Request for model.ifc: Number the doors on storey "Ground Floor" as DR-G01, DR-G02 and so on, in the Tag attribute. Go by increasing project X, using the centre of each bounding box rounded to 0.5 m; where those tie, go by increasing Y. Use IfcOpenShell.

First a look at what the model holds.

```python
import ifcopenshell
import ifcopenshell.util.element
import ifcopenshell.util.placement

model = ifcopenshell.open("model.ifc")
print(model.schema)
storey = next(s for s in model.by_type("IfcBuildingStorey") if s.Name == "Ground Floor")
doors = [e for e in ifcopenshell.util.element.get_decomposition(storey) if e.is_a("IfcDoor")]
for e in sorted(doors, key=lambda e: e.id()):
    origin = ifcopenshell.util.placement.get_local_placement(e.ObjectPlacement)[:3, 3]
    print(e.id(), e.Tag, e.Name, origin.round(2) + 0.0, sep=" | ")
```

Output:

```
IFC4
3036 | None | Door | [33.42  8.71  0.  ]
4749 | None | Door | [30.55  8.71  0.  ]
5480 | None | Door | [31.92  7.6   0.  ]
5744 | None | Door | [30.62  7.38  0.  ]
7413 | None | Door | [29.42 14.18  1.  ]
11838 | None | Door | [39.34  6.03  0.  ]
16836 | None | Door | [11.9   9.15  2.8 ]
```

```python
import ifcopenshell
import ifcopenshell.geom
import ifcopenshell.util.element
import ifcopenshell.util.shape

model = ifcopenshell.open("model.ifc")
settings = ifcopenshell.geom.settings()
settings.set("use-world-coords", True)


def centre(element):
    shape = ifcopenshell.geom.create_shape(settings, element)
    return ifcopenshell.util.shape.get_bbox_centroid(shape.geometry)


storey = next(s for s in model.by_type("IfcBuildingStorey") if s.Name == "Ground Floor")
doors = [e for e in ifcopenshell.util.element.get_decomposition(storey) if e.is_a("IfcDoor")]

# Insertion points can sit at a corner or the storey origin, so sort by the geometry (in metres).
centres = {e: centre(e) for e in doors}
doors.sort(key=lambda e: (round(centres[e][0] / 0.5), centres[e][1]))

for i, e in enumerate(doors, start=1):
    number = f"DR-G{i:02d}"
    e.Tag = number
    print(e.id(), number)

model.write("model_rev.ifc")
```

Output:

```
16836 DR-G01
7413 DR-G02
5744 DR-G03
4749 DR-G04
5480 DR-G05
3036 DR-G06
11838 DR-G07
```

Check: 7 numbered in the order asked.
